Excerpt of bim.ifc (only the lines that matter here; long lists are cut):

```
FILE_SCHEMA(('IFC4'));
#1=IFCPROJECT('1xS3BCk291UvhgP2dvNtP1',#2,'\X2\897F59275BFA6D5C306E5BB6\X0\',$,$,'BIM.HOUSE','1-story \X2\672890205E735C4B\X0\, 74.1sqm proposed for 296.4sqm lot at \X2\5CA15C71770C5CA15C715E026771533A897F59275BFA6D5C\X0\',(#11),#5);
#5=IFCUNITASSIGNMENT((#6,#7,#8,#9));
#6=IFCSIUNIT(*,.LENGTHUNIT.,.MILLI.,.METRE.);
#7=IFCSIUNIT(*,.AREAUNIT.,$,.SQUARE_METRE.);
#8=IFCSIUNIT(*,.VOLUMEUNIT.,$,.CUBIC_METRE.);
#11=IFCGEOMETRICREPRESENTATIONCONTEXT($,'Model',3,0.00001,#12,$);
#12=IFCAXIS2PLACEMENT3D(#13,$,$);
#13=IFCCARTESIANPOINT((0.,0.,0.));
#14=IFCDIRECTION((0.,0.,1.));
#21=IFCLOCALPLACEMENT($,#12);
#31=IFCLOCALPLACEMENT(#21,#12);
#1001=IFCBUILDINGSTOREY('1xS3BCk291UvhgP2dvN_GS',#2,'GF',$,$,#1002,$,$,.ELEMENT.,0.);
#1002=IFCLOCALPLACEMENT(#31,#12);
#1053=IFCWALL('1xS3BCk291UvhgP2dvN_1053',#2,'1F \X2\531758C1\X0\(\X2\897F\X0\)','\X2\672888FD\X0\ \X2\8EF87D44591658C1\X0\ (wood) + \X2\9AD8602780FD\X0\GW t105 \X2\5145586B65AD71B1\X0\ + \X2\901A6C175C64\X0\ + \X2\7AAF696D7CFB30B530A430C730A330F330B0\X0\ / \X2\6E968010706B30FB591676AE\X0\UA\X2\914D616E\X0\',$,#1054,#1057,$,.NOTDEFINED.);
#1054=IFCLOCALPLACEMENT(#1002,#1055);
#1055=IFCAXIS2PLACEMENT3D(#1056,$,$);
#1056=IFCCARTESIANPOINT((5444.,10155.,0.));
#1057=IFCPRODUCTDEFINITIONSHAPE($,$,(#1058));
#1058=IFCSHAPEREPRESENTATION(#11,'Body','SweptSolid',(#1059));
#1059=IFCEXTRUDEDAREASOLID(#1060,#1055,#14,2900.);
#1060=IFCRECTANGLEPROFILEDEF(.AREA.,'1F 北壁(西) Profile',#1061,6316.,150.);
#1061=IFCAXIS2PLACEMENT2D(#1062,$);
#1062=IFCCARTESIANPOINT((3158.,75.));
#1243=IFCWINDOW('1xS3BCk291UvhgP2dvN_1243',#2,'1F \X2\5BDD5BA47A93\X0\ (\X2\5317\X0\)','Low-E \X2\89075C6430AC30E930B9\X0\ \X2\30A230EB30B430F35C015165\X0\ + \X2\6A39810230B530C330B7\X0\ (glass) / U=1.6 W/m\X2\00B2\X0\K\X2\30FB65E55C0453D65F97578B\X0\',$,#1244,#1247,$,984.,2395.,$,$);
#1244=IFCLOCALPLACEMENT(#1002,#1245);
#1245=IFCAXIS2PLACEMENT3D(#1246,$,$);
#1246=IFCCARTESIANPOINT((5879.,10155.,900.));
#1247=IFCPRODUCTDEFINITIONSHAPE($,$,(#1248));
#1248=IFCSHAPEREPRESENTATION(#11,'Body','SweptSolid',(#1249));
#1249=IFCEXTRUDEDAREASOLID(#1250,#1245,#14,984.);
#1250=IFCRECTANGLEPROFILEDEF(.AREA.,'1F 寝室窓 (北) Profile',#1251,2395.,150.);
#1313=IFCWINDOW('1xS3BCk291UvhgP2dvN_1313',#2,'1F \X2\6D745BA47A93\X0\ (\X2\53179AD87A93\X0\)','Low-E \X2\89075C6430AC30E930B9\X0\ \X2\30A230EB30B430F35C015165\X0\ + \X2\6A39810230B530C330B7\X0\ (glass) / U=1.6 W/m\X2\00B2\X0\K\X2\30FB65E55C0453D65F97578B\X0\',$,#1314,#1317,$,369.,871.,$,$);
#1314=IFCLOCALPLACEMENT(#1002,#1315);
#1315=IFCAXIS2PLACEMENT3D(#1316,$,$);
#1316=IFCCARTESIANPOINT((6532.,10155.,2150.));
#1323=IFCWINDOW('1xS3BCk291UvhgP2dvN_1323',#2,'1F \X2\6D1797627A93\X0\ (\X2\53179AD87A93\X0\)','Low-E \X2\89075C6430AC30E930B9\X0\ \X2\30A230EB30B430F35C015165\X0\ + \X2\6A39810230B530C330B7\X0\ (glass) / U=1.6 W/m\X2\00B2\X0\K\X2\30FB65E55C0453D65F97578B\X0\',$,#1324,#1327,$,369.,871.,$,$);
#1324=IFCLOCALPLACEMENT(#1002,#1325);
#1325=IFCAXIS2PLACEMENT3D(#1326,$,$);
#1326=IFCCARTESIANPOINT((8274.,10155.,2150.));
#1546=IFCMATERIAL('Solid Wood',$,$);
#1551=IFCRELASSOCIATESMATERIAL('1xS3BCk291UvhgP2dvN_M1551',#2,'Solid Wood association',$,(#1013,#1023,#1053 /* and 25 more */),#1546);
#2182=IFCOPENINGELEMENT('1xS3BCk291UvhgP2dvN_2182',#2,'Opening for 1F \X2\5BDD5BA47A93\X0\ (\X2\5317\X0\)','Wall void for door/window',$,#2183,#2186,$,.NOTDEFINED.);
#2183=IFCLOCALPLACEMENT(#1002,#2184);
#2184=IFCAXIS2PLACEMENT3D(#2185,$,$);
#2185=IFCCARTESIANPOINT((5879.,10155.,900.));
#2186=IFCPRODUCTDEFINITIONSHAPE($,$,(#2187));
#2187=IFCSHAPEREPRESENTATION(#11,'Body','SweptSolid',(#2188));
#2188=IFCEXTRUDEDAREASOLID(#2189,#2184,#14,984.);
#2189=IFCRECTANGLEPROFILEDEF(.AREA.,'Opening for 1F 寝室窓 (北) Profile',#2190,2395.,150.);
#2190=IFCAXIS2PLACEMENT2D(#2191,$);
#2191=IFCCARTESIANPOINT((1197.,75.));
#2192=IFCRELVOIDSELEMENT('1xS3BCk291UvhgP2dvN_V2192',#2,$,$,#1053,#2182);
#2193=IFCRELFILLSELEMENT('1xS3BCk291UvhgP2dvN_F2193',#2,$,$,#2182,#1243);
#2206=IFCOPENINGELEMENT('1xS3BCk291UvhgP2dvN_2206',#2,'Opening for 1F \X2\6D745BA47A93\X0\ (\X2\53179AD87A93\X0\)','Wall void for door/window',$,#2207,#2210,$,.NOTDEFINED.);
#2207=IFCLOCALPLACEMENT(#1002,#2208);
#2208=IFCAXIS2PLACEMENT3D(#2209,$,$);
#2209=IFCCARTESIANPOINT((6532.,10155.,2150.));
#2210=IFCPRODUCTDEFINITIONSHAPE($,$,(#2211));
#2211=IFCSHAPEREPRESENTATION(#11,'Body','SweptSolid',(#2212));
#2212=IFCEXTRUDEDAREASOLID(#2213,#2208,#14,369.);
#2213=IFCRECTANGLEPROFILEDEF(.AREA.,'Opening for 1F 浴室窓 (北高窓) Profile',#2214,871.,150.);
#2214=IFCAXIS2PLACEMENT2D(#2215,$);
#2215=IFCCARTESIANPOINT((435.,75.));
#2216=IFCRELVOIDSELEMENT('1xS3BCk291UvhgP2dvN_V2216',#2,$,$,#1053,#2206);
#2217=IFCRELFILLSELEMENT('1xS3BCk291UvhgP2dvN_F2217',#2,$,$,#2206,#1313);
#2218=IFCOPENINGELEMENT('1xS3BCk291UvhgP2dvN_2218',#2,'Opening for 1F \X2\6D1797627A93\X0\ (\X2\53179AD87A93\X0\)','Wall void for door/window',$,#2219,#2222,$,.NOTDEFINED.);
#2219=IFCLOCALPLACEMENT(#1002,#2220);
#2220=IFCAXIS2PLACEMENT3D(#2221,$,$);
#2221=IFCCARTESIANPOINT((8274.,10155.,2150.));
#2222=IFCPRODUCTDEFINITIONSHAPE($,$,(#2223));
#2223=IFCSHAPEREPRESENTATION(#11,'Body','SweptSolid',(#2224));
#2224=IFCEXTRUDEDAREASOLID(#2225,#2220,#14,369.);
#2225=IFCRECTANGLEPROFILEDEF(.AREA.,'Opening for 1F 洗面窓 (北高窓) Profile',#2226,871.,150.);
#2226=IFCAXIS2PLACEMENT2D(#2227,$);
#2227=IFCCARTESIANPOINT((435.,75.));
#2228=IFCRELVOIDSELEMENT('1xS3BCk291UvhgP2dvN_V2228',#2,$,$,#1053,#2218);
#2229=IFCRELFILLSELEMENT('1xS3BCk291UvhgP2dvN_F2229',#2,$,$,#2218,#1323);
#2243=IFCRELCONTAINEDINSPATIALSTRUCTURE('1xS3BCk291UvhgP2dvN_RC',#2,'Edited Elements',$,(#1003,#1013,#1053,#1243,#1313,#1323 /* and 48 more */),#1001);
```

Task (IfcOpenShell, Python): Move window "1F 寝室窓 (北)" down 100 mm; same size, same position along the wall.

```python
import numpy as np
import ifcopenshell
import ifcopenshell.api.geometry
import ifcopenshell.util.placement
import ifcopenshell.util.unit

model = ifcopenshell.open("bim.ifc")
unit_scale = ifcopenshell.util.unit.calculate_unit_scale(model)

window = model.by_guid("1xS3BCk291UvhgP2dvN_1243")
opening = window.FillsVoids[0].RelatingOpeningElement
dz = -0.1 / unit_scale

shift = np.array([0.0, 0.0, dz])
# The window is not placed relative to its opening, so move both.
for product in (opening, window):
    matrix = ifcopenshell.util.placement.get_local_placement(product.ObjectPlacement)
    matrix[:3, 3] += shift
    ifcopenshell.api.geometry.edit_object_placement(model, product=product, matrix=matrix, is_si=False)

print(f"moved by {dz * unit_scale:+.3f} m")

model.write("bim_v2.ifc")
```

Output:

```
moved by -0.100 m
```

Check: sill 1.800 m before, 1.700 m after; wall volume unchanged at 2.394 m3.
